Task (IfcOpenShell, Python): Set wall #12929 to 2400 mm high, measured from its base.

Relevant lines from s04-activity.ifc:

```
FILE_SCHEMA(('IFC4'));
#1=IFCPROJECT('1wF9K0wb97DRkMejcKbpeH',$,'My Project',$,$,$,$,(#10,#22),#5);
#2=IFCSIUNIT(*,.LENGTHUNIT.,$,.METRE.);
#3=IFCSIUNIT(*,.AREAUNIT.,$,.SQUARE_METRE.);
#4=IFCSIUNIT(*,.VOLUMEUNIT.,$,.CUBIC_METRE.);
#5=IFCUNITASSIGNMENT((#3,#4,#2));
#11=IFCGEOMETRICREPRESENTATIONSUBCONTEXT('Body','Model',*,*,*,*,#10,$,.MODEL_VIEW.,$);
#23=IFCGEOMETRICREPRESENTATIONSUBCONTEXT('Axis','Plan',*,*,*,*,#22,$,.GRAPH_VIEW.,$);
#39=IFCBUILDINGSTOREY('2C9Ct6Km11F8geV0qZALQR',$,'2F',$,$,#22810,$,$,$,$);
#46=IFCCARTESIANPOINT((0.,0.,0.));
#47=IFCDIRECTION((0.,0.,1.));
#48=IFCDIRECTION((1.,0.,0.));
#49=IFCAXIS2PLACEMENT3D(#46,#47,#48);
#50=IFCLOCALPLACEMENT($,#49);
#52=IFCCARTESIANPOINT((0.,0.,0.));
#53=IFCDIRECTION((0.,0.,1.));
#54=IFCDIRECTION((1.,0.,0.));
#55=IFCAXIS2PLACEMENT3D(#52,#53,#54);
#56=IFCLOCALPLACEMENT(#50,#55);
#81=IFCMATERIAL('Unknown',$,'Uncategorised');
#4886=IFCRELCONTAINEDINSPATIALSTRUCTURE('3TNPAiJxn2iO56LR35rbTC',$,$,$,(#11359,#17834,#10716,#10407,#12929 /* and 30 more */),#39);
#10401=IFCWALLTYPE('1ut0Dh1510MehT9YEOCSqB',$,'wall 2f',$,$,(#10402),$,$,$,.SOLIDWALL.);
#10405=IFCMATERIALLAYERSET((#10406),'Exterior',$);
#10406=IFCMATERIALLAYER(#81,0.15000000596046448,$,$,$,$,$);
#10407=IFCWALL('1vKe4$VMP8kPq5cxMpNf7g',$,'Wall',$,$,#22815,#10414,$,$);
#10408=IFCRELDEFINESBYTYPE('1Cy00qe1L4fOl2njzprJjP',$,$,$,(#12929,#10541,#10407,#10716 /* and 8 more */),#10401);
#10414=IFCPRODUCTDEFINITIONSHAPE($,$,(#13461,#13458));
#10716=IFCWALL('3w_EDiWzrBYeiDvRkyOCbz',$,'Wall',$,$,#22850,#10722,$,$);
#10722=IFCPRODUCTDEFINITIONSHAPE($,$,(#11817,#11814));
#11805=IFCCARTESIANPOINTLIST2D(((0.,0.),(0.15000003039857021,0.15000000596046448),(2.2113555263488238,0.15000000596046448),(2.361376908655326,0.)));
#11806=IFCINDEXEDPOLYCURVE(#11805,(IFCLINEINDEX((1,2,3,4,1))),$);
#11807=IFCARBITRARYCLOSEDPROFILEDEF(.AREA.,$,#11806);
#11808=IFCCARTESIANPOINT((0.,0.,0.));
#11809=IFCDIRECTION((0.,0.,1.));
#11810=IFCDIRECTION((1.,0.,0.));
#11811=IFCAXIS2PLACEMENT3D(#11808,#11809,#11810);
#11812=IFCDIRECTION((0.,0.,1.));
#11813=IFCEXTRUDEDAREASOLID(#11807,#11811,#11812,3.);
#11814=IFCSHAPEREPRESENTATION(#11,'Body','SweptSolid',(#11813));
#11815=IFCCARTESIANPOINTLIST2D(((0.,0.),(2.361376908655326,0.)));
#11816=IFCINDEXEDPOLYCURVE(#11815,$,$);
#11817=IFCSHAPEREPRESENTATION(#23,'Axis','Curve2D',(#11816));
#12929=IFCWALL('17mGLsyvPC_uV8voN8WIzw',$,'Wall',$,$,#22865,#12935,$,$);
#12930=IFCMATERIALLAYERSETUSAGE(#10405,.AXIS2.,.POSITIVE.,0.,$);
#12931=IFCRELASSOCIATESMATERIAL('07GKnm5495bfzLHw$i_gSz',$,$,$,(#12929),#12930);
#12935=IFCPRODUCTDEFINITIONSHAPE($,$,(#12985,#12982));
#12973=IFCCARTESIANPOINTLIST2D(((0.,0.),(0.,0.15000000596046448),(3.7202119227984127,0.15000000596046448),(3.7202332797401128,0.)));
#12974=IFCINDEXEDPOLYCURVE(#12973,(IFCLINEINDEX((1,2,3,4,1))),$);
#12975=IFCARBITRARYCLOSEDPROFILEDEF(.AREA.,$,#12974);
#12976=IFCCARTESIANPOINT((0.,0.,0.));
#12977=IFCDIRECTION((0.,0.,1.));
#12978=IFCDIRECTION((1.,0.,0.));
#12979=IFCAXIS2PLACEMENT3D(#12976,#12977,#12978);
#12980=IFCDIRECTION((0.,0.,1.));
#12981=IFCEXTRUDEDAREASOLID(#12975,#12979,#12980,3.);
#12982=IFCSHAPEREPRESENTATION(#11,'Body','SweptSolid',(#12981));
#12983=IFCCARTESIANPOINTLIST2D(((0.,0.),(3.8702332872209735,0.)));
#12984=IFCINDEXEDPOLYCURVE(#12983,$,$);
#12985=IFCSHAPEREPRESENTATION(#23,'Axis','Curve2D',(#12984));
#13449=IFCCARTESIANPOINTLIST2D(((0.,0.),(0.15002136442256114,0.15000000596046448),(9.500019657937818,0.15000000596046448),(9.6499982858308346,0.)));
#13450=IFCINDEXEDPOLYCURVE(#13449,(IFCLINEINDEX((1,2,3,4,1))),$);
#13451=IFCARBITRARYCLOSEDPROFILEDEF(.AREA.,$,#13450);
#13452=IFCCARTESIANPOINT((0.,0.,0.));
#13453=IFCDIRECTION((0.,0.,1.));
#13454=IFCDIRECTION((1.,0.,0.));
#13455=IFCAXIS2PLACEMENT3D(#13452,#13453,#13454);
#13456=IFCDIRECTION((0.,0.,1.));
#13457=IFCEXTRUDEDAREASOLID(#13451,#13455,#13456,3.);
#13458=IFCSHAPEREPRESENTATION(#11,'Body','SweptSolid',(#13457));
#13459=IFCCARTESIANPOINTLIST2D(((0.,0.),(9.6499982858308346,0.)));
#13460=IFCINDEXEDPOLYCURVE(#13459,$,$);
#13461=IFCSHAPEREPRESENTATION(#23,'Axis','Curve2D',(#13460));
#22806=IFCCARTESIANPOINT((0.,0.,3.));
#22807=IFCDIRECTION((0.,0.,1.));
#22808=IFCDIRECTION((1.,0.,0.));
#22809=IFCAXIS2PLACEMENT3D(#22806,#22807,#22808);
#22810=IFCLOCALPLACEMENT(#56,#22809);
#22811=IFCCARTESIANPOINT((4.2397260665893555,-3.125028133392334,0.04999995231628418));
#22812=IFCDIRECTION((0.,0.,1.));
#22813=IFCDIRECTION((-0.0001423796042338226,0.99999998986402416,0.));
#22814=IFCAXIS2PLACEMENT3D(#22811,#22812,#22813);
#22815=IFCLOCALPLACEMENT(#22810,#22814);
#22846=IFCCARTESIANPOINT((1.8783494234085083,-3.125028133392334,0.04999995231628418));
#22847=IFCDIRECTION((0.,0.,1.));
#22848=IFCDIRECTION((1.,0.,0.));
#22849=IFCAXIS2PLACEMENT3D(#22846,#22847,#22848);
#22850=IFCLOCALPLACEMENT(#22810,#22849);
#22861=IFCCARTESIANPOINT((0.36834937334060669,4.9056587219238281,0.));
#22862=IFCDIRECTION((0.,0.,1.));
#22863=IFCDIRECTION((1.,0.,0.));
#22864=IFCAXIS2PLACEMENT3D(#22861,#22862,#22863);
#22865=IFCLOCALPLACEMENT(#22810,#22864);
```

```python
import ifcopenshell
import ifcopenshell.geom
import ifcopenshell.util.representation
import ifcopenshell.util.shape

model = ifcopenshell.open("s04-activity.ifc")
settings = ifcopenshell.geom.settings()


def volume(element):
    """Net volume in cubic metres, openings subtracted."""
    shape = ifcopenshell.geom.create_shape(settings, element)
    return ifcopenshell.util.shape.get_volume(shape.geometry)


wall = model.by_id(12929)
before = volume(wall)

body = ifcopenshell.util.representation.get_representation(wall, "Model", "Body")
solid = body.Items[0]
old_height = solid.Depth
solid.Depth = 2.4
after = volume(wall)

print(f"height {old_height:g} -> {solid.Depth:g}, volume {before:.3f} -> {after:.3f} m3")

model.write("s04-activity_rev.ifc")
```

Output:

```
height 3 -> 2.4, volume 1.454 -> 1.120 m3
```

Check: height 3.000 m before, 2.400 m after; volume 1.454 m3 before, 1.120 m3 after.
